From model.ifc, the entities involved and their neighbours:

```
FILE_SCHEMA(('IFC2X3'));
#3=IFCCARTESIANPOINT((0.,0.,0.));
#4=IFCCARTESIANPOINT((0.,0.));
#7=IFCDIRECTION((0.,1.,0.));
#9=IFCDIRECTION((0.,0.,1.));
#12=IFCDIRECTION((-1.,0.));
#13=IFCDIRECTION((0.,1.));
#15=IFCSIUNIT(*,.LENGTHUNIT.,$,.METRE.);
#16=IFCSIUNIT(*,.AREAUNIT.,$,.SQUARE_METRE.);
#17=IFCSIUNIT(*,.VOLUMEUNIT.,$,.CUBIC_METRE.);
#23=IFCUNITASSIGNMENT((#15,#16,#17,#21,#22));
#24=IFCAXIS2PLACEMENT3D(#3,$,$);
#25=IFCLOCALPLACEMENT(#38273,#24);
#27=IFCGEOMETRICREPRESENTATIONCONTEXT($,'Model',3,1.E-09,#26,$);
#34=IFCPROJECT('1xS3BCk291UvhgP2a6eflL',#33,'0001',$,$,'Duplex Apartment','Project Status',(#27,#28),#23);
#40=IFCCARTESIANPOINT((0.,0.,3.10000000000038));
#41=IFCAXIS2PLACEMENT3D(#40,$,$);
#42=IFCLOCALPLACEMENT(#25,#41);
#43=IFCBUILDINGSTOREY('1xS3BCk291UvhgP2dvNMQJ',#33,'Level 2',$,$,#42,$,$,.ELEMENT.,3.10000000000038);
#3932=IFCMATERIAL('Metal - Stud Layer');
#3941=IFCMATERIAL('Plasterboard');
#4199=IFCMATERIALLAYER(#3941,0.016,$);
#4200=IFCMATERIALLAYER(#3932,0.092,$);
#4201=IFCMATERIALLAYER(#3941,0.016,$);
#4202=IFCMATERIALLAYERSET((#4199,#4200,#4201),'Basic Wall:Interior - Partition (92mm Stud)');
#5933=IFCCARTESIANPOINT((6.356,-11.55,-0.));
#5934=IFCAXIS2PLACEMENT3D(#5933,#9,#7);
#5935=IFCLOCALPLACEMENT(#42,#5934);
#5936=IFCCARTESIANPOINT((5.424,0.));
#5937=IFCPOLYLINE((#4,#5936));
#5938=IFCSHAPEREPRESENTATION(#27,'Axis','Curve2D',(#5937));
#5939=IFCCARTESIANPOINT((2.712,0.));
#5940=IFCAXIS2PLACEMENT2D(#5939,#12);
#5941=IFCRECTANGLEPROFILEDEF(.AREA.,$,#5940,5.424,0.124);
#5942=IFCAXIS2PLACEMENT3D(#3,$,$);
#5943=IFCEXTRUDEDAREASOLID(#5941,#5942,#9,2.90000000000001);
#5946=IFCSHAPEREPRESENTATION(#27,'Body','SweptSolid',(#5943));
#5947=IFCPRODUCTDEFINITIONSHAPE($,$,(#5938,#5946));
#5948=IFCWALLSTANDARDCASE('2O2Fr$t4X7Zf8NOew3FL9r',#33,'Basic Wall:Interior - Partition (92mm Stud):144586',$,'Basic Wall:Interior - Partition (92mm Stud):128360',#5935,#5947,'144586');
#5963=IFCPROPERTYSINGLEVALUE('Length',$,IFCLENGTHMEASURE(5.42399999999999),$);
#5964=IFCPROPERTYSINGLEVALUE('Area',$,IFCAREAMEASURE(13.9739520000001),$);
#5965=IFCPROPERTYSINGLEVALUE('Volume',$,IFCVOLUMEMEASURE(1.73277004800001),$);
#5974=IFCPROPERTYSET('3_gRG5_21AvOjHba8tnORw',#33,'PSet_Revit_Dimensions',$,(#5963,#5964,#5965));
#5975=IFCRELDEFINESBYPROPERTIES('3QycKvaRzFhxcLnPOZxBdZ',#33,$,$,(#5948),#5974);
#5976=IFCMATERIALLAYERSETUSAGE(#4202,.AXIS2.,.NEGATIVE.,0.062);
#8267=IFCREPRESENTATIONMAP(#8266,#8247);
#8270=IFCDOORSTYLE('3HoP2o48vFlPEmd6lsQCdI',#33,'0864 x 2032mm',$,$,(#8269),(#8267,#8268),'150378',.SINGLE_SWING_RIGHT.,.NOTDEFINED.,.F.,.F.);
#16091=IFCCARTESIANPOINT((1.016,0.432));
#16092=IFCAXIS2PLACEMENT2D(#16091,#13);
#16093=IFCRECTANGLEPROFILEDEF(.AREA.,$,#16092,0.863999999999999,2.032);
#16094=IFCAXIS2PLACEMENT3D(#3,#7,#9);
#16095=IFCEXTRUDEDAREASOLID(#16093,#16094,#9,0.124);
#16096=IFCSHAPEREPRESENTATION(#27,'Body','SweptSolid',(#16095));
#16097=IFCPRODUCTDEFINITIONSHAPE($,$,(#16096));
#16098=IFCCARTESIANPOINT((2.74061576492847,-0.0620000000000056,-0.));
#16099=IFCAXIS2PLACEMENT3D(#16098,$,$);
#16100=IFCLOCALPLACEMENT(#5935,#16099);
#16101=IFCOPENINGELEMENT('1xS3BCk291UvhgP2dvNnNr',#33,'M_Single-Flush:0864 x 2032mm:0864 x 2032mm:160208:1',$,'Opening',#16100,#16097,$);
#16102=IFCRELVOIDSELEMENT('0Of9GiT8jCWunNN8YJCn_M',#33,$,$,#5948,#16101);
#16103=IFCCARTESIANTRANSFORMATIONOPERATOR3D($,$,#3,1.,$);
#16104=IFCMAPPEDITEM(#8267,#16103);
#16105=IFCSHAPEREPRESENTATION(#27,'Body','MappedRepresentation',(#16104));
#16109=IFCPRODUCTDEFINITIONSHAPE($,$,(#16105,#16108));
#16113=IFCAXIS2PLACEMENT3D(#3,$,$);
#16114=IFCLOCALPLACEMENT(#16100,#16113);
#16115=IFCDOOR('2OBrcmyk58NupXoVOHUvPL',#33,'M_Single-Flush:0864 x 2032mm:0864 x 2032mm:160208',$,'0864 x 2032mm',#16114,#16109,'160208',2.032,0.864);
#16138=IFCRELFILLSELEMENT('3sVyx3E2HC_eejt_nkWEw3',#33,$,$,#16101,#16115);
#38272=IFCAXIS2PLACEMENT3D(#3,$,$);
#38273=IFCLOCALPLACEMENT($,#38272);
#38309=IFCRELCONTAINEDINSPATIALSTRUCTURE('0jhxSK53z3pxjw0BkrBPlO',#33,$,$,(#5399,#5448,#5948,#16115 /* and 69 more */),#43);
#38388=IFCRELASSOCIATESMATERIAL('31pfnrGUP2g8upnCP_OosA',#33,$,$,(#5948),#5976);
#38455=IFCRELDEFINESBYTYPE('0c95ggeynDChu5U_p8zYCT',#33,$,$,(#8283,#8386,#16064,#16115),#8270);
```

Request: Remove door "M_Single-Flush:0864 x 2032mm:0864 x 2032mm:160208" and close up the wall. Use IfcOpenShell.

```python
import ifcopenshell
import ifcopenshell.api.feature
import ifcopenshell.api.pset
import ifcopenshell.api.root
import ifcopenshell.geom
import ifcopenshell.util.element
import ifcopenshell.util.shape
import ifcopenshell.util.unit

model = ifcopenshell.open("model.ifc")
area_scale = ifcopenshell.util.unit.calculate_unit_scale(model, "AREAUNIT")
volume_scale = ifcopenshell.util.unit.calculate_unit_scale(model, "VOLUMEUNIT")
settings = ifcopenshell.geom.settings()


def volume(element):
    """Net volume in cubic metres, openings subtracted."""
    shape = ifcopenshell.geom.create_shape(settings, element)
    return ifcopenshell.util.shape.get_volume(shape.geometry)


door = model.by_guid("2OBrcmyk58NupXoVOHUvPL")
opening = door.FillsVoids[0].RelatingOpeningElement
wall = opening.VoidsElements[0].RelatingBuildingElement
before = volume(wall)

ifcopenshell.api.root.remove_product(model, product=door)
ifcopenshell.api.feature.remove_feature(model, feature=opening)

after = volume(wall)
thickness = 0.124  # wall thickness in metres

# Update the wall's stored quantities.
pset = model.by_id(ifcopenshell.util.element.get_pset(wall, "PSet_Revit_Dimensions", should_inherit=False)["id"])
ifcopenshell.api.pset.edit_pset(model, pset=pset, properties={
    "Area": model.create_entity("IfcAreaMeasure", after / thickness / area_scale),
    "Volume": model.create_entity("IfcVolumeMeasure", after / volume_scale),
})

print(f"wall volume {before:.3f} -> {after:.3f} m3")

model.write("model_v2.ifc")
```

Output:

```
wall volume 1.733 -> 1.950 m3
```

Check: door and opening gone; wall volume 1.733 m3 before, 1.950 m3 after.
